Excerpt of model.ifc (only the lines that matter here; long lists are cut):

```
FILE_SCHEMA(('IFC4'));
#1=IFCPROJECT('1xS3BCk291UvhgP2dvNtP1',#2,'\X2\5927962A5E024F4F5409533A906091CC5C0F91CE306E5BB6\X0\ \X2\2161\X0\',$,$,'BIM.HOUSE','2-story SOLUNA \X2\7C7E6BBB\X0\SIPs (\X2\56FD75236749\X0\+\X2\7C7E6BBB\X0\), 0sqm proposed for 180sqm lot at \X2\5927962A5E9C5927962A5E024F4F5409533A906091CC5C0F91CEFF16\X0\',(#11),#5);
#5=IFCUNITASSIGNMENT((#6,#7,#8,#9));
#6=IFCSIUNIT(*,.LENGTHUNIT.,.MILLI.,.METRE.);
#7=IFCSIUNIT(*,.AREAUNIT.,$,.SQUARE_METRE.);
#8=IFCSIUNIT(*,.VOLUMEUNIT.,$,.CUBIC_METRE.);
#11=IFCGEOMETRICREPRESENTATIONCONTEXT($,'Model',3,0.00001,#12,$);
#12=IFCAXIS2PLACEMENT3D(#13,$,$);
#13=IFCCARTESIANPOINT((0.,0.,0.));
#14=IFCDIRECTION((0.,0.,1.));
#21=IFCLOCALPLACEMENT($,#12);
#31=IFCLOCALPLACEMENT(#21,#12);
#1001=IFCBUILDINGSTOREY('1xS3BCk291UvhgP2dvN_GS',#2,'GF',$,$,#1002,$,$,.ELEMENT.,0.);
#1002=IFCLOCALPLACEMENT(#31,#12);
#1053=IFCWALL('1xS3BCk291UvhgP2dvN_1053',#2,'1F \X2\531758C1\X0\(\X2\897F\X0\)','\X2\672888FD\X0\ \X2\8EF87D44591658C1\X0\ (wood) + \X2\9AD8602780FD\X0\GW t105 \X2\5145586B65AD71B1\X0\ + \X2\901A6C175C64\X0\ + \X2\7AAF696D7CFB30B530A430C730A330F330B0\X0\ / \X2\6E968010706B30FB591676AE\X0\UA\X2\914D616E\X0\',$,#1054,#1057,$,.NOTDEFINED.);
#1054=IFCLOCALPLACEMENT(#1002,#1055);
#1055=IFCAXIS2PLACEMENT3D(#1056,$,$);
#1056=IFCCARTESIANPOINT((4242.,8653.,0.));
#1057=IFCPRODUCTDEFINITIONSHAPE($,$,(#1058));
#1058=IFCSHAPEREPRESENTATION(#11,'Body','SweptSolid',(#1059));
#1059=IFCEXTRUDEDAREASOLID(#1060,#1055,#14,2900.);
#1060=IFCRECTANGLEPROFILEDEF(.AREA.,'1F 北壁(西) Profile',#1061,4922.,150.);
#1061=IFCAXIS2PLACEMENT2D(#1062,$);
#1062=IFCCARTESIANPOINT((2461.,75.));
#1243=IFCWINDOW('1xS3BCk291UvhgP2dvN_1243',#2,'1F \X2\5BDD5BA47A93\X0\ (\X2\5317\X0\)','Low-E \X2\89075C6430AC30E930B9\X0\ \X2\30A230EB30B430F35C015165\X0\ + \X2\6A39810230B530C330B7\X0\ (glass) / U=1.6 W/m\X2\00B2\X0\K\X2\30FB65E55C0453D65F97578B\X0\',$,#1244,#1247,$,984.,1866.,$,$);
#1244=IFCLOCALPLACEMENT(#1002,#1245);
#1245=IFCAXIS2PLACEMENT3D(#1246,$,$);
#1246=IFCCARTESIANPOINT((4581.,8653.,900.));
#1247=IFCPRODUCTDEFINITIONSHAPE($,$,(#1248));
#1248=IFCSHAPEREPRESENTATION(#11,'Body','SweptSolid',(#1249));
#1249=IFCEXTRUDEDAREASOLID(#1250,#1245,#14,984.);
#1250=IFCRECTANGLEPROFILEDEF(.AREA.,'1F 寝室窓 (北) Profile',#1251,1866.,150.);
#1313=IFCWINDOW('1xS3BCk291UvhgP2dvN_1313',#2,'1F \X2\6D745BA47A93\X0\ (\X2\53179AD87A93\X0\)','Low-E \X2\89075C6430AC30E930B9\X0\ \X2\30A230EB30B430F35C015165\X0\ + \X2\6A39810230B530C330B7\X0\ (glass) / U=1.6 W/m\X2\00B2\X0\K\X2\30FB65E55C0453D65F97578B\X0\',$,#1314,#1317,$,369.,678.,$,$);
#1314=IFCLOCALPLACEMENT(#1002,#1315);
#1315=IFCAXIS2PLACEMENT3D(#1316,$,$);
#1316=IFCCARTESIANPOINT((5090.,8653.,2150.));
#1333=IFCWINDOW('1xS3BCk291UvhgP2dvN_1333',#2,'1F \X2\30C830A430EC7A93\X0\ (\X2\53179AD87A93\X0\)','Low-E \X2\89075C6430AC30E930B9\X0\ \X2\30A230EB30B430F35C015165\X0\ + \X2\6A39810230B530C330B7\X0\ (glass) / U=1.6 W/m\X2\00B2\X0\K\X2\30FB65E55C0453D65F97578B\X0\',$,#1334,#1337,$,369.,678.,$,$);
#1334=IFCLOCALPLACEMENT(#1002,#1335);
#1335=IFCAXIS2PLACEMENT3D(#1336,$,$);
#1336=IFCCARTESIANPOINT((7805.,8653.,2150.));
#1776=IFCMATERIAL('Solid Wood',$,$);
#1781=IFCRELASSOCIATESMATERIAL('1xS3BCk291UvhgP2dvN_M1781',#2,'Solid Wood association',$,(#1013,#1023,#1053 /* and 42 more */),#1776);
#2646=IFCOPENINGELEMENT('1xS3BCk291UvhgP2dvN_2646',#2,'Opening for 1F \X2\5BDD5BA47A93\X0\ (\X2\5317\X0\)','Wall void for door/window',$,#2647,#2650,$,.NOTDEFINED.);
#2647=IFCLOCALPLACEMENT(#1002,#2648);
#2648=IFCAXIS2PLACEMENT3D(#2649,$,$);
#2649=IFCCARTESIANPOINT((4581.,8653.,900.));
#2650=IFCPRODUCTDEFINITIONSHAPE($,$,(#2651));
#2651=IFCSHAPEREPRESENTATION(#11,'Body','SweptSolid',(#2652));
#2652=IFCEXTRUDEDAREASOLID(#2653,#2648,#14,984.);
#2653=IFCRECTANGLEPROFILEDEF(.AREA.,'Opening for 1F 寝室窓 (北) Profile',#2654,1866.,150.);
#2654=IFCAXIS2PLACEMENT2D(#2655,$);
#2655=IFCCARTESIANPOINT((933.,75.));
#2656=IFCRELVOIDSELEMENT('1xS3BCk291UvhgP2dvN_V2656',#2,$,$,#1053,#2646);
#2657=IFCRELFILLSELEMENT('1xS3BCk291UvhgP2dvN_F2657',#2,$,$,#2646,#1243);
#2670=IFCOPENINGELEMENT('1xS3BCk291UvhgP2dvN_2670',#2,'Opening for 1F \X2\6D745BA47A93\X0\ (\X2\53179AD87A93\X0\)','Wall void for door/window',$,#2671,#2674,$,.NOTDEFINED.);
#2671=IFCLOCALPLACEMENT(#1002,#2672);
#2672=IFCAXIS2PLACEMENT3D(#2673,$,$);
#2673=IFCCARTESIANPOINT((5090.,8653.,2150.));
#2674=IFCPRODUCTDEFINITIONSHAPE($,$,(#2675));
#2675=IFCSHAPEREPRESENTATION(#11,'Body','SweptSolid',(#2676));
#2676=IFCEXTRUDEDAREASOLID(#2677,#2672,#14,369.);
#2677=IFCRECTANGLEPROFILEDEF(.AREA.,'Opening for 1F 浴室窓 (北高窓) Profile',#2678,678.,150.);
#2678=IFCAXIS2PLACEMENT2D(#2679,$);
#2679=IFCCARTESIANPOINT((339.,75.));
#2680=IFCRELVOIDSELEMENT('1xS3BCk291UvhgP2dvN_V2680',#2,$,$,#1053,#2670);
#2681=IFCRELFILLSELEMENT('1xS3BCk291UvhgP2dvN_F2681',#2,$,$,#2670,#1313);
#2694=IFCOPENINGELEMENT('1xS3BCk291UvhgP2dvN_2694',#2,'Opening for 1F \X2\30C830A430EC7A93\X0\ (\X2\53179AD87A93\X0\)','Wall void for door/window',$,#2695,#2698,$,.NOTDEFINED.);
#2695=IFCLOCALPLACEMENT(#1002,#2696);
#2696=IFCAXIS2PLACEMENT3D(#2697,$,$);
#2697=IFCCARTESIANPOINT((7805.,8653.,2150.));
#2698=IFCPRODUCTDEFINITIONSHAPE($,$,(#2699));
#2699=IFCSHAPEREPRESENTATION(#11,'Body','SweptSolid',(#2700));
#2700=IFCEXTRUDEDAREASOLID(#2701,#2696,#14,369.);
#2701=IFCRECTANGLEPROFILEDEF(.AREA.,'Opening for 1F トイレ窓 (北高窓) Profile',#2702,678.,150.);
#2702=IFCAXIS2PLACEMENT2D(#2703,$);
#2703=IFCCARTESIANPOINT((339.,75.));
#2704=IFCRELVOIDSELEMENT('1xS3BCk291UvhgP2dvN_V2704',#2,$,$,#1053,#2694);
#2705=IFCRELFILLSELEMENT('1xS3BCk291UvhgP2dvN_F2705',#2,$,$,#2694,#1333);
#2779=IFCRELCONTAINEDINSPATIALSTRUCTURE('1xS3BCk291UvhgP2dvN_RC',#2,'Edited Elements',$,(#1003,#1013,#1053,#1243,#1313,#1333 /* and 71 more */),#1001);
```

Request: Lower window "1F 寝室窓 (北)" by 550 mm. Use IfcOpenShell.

```python
import numpy as np
import ifcopenshell
import ifcopenshell.api.geometry
import ifcopenshell.util.placement
import ifcopenshell.util.unit

model = ifcopenshell.open("model.ifc")
unit_scale = ifcopenshell.util.unit.calculate_unit_scale(model)

window = model.by_id(1243)
opening = window.FillsVoids[0].RelatingOpeningElement
dz = -550.0

shift = np.array([0.0, 0.0, dz])
# The window is not placed relative to its opening, so move both.
for product in (opening, window):
    matrix = ifcopenshell.util.placement.get_local_placement(product.ObjectPlacement)
    matrix[:3, 3] += shift
    ifcopenshell.api.geometry.edit_object_placement(model, product=product, matrix=matrix, is_si=False)

print(f"moved by {dz * unit_scale:+.3f} m")

model.write("model_rev.ifc")
```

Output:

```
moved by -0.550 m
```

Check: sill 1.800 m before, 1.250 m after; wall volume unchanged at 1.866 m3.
